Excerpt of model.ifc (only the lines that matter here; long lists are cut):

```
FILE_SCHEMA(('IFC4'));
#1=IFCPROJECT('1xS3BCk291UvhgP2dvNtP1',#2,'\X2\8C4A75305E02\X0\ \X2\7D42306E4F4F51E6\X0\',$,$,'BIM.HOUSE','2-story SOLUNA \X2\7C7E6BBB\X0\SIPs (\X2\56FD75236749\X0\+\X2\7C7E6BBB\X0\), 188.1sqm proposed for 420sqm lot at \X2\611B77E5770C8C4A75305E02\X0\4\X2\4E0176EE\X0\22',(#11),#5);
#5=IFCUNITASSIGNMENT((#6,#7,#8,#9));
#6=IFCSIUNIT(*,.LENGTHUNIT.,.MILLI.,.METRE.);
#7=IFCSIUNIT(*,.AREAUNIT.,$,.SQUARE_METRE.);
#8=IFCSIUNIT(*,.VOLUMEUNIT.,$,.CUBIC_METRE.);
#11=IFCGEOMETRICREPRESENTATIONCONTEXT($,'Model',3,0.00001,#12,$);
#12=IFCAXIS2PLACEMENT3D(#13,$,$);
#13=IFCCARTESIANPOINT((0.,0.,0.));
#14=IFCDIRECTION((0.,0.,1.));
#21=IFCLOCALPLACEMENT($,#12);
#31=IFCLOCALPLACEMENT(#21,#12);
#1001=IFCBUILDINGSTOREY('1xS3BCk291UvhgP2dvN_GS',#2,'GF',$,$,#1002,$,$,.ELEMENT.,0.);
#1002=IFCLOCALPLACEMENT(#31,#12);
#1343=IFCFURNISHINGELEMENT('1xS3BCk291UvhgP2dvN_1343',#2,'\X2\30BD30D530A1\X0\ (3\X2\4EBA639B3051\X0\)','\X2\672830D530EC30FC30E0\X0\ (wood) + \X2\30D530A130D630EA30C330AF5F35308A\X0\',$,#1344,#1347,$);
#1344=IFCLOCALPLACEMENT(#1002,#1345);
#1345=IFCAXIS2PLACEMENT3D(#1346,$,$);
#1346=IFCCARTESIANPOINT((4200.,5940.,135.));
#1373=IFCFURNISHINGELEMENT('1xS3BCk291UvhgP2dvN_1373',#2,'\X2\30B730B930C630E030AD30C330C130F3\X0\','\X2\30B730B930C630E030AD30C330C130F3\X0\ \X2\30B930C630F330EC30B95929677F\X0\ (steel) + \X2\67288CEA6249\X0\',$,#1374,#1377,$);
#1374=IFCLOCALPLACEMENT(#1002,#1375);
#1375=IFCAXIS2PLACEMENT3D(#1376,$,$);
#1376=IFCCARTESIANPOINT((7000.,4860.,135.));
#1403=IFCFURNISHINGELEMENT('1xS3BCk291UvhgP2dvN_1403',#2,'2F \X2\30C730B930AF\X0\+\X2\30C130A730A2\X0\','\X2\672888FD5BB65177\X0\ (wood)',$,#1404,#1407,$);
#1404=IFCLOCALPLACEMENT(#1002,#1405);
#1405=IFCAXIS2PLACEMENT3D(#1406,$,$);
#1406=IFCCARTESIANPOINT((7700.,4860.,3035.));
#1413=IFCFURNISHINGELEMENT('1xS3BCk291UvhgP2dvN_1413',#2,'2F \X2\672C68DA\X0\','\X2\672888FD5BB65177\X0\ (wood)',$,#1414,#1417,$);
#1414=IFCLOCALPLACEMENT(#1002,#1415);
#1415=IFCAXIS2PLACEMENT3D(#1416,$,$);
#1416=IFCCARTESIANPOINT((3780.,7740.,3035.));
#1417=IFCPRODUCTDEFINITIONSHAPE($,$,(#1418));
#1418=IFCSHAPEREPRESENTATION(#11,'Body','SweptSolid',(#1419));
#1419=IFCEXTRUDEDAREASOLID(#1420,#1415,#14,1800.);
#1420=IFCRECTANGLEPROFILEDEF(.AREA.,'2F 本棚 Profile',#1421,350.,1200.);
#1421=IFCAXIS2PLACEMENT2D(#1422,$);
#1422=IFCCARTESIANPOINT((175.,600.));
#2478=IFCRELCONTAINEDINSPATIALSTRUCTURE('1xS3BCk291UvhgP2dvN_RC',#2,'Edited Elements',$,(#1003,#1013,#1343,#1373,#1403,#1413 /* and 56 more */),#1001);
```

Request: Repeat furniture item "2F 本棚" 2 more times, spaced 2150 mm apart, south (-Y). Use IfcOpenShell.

```python
import numpy as np
import ifcopenshell
import ifcopenshell.api.geometry
import ifcopenshell.api.root
import ifcopenshell.util.element
import ifcopenshell.util.placement
import ifcopenshell.util.unit

model = ifcopenshell.open("model.ifc")
unit_scale = ifcopenshell.util.unit.calculate_unit_scale(model)


def reuse_history(source, copy):
    """copy_class also copies each property set's owner history, people and application; keep the originals."""
    for rel in copy.IsDefinedBy:
        if rel.is_a("IfcRelDefinesByProperties") and (history := rel.RelatingPropertyDefinition.OwnerHistory):
            rel.RelatingPropertyDefinition.OwnerHistory = source.OwnerHistory
            ifcopenshell.util.element.remove_deep2(model, history)


source = model.by_guid("1xS3BCk291UvhgP2dvN_1413")
base = ifcopenshell.util.placement.get_local_placement(source.ObjectPlacement)
step = np.array([0.0, -1.0, 0.0]) * 2.15 / unit_scale

for i in range(1, 3):
    copy = ifcopenshell.api.root.copy_class(model, product=source)
    copy.Representation = ifcopenshell.util.element.copy_deep(
        model, source.Representation, exclude=["IfcGeometricRepresentationContext", "IfcRepresentationMap"]
    )
    reuse_history(source, copy)
    matrix = base.copy()
    matrix[:3, 3] += i * step
    print("added at", matrix[:3, 3].round(3) + 0.0)
    ifcopenshell.api.geometry.edit_object_placement(model, product=copy, matrix=matrix, is_si=False)

model.write("model_v2.ifc")
```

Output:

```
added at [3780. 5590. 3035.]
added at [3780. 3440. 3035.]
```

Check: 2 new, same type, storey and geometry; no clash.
